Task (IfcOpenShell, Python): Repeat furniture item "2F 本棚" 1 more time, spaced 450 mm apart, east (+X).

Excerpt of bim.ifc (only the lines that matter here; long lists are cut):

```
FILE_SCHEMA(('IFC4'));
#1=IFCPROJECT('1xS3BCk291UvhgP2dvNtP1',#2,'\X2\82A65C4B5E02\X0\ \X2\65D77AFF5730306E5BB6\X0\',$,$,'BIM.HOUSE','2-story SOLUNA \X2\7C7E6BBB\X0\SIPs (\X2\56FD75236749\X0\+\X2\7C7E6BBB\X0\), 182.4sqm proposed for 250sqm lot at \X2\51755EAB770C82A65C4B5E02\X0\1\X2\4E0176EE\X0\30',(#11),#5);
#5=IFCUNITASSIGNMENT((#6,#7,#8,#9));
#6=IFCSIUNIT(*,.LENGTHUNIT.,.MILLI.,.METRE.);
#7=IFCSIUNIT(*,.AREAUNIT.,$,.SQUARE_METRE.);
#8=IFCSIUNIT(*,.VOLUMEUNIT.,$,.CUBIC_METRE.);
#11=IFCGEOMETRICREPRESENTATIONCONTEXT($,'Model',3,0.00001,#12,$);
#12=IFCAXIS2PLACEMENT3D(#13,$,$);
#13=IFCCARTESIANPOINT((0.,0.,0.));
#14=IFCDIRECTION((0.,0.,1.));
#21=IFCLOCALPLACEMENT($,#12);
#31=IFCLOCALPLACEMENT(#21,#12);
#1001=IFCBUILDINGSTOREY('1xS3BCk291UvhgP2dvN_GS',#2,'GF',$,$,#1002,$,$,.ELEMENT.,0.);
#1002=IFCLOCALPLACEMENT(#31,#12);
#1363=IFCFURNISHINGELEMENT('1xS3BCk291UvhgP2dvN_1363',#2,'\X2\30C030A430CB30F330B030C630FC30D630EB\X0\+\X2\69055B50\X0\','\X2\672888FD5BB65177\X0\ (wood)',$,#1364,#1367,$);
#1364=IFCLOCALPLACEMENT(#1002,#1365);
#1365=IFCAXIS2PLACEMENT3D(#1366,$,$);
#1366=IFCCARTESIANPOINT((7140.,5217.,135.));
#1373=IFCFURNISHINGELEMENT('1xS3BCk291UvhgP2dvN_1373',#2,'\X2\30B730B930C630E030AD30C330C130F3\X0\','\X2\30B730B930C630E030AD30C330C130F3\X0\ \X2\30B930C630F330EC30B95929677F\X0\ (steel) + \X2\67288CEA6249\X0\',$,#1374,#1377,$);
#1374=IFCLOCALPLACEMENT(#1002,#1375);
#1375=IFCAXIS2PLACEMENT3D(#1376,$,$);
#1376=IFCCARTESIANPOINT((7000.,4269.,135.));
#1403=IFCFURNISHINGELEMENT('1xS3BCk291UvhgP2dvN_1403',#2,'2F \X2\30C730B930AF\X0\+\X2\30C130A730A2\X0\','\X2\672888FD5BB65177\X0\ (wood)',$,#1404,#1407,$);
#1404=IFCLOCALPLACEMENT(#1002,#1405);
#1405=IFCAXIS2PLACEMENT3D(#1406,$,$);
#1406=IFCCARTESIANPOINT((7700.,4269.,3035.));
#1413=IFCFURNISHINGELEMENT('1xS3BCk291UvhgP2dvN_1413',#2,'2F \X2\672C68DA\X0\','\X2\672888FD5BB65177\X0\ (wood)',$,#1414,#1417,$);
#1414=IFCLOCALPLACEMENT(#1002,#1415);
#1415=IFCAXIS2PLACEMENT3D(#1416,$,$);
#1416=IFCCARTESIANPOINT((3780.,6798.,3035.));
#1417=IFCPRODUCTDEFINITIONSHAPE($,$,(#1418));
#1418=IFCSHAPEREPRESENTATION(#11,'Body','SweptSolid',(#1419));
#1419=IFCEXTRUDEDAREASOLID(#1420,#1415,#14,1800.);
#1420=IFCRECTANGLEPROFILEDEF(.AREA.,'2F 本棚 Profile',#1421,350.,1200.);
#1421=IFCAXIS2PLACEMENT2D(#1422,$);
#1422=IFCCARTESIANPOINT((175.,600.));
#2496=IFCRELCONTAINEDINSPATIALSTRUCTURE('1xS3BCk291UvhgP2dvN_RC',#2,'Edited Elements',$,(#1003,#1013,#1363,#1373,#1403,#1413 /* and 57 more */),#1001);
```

```python
import numpy as np
import ifcopenshell
import ifcopenshell.api.geometry
import ifcopenshell.api.root
import ifcopenshell.util.element
import ifcopenshell.util.placement

model = ifcopenshell.open("bim.ifc")


def reuse_history(source, copy):
    """copy_class also copies each property set's owner history, people and application; keep the originals."""
    for rel in copy.IsDefinedBy:
        if rel.is_a("IfcRelDefinesByProperties") and (history := rel.RelatingPropertyDefinition.OwnerHistory):
            rel.RelatingPropertyDefinition.OwnerHistory = source.OwnerHistory
            ifcopenshell.util.element.remove_deep2(model, history)


source = model.by_guid("1xS3BCk291UvhgP2dvN_1413")
base = ifcopenshell.util.placement.get_local_placement(source.ObjectPlacement)
step = np.array([1.0, 0.0, 0.0]) * 450.0

for i in range(1, 2):
    copy = ifcopenshell.api.root.copy_class(model, product=source)
    copy.Representation = ifcopenshell.util.element.copy_deep(
        model, source.Representation, exclude=["IfcGeometricRepresentationContext", "IfcRepresentationMap"]
    )
    reuse_history(source, copy)
    matrix = base.copy()
    matrix[:3, 3] += i * step
    print("added at", matrix[:3, 3].round(3) + 0.0)
    ifcopenshell.api.geometry.edit_object_placement(model, product=copy, matrix=matrix, is_si=False)

model.write("bim_rev.ifc")
```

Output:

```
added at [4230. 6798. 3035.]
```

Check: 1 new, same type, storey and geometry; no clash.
